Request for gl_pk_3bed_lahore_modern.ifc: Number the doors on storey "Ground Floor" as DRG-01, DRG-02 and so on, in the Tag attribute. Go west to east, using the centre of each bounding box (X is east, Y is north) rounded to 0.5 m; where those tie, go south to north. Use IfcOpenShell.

First a look at what the model holds.

```python
import ifcopenshell
import ifcopenshell.util.element
import ifcopenshell.util.placement

model = ifcopenshell.open("gl_pk_3bed_lahore_modern.ifc")
print(model.schema)
storey = next(s for s in model.by_type("IfcBuildingStorey") if s.Name == "Ground Floor")
doors = [e for e in ifcopenshell.util.element.get_decomposition(storey) if e.is_a("IfcDoor")]
for e in sorted(doors, key=lambda e: e.id()):
    origin = ifcopenshell.util.placement.get_local_placement(e.ObjectPlacement)[:3, 3]
    print(e.id(), e.Tag, e.Name, origin.round(2) + 0.0, sep=" | ")
```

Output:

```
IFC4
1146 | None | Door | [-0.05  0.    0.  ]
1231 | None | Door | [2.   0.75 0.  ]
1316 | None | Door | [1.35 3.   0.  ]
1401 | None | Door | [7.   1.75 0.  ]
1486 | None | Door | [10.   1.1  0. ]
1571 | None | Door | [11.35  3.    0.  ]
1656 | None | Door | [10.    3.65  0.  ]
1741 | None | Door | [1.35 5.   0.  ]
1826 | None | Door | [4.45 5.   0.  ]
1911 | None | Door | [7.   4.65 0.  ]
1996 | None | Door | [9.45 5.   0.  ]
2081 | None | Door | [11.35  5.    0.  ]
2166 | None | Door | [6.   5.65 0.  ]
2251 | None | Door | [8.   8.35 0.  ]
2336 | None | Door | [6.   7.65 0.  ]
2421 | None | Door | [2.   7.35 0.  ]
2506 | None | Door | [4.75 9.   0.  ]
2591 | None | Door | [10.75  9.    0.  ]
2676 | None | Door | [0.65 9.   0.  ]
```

```python
import ifcopenshell
import ifcopenshell.geom
import ifcopenshell.util.element
import ifcopenshell.util.shape

model = ifcopenshell.open("gl_pk_3bed_lahore_modern.ifc")
settings = ifcopenshell.geom.settings()
settings.set("use-world-coords", True)


def centre(element):
    shape = ifcopenshell.geom.create_shape(settings, element)
    return ifcopenshell.util.shape.get_bbox_centroid(shape.geometry)


storey = next(s for s in model.by_type("IfcBuildingStorey") if s.Name == "Ground Floor")
doors = [e for e in ifcopenshell.util.element.get_decomposition(storey) if e.is_a("IfcDoor")]

# Insertion points can sit at a corner or the storey origin, so sort by the geometry (in metres).
centres = {e: centre(e) for e in doors}
doors.sort(key=lambda e: (round(centres[e][0] / 0.5), centres[e][1]))

for i, e in enumerate(doors, start=1):
    number = f"DRG-{i:02d}"
    e.Tag = number
    print(e.id(), number)

model.write("gl_pk_3bed_lahore_modern_updated.ifc")
```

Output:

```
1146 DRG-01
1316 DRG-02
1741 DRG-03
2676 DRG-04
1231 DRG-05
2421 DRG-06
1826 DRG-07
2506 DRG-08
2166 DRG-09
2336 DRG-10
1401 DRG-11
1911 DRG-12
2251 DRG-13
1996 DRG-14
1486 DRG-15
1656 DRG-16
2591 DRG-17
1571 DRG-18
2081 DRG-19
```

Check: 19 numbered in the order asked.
